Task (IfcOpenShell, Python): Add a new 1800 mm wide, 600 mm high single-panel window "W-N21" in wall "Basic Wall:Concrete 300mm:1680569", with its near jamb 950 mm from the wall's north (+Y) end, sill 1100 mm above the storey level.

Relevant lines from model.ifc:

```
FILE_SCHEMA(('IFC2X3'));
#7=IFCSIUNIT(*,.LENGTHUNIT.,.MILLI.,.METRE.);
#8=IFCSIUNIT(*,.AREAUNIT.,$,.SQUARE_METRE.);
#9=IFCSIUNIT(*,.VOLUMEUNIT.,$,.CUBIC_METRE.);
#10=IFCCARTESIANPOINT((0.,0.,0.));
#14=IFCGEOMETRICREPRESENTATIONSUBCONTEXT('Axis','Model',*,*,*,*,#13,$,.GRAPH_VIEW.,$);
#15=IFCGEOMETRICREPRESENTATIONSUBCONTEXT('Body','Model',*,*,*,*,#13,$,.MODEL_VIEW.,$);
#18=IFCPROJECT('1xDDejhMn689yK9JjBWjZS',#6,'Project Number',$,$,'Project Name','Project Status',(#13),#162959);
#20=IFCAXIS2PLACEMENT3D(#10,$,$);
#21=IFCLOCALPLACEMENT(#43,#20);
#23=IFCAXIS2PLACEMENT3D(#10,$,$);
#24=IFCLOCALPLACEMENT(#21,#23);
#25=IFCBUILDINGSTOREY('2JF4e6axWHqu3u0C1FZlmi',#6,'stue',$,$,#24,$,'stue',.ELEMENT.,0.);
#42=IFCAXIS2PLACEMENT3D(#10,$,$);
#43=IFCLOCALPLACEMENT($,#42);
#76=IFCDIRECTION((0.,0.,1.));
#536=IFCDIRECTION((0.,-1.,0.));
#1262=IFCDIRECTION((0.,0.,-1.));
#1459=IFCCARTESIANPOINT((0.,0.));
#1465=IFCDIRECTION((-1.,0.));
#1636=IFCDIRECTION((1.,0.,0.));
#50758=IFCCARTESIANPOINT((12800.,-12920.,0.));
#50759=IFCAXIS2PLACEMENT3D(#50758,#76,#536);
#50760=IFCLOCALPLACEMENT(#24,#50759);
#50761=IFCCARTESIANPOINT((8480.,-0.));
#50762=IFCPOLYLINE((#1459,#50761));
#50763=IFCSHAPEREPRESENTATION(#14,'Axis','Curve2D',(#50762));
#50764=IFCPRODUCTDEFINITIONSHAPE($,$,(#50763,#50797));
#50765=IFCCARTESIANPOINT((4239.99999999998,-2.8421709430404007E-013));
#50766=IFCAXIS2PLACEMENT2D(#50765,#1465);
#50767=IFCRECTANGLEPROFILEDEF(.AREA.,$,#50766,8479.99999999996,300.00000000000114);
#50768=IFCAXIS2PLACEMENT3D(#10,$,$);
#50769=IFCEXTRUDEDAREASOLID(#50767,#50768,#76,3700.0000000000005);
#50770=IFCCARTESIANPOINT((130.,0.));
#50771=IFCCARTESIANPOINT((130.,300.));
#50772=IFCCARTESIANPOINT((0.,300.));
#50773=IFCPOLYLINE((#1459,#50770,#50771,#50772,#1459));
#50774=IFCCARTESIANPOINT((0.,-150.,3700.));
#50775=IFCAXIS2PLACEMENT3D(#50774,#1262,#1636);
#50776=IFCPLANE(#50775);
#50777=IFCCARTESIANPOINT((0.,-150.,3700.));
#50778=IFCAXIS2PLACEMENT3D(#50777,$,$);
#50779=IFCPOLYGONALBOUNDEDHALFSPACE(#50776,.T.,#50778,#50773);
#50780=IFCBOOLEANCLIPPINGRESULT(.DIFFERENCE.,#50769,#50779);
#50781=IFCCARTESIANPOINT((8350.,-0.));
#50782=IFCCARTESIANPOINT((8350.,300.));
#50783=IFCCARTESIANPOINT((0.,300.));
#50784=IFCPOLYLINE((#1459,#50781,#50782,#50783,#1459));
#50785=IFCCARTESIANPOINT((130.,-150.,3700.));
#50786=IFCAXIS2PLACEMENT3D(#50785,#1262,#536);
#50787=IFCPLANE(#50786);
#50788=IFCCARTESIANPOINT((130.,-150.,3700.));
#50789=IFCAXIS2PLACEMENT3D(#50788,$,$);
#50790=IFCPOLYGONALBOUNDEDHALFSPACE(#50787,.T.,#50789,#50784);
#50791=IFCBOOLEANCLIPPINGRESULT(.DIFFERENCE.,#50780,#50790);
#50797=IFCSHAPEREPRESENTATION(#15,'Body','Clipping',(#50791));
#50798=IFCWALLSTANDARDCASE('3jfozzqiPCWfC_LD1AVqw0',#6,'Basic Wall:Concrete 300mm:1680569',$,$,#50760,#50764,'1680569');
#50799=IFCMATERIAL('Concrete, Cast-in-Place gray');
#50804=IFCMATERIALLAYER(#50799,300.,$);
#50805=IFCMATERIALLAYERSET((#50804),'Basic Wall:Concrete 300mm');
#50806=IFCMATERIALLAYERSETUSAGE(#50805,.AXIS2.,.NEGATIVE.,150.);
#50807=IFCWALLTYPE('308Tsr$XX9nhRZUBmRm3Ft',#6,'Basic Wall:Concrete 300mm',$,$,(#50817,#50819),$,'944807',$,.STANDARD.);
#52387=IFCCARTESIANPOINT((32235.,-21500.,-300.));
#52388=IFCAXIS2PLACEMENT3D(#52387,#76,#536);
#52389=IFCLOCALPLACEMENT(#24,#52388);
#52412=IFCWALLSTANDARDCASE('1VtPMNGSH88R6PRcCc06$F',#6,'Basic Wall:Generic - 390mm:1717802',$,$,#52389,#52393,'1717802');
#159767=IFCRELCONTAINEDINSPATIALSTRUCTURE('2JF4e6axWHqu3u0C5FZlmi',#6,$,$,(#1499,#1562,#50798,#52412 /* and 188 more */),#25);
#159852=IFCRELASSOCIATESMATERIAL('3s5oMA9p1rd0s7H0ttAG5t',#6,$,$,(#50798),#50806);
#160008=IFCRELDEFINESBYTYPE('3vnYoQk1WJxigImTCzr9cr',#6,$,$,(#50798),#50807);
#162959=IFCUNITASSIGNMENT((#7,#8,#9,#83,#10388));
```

```python
import numpy as np
import ifcopenshell
import ifcopenshell.api.feature
import ifcopenshell.api.geometry
import ifcopenshell.api.root
import ifcopenshell.api.spatial
import ifcopenshell.api.type
import ifcopenshell.geom
import ifcopenshell.util.element
import ifcopenshell.util.placement
import ifcopenshell.util.representation
import ifcopenshell.util.shape
import ifcopenshell.util.unit

model = ifcopenshell.open("model.ifc")
unit_scale = ifcopenshell.util.unit.calculate_unit_scale(model)
settings = ifcopenshell.geom.settings()


def volume(element):
    """Net volume in cubic metres, openings subtracted."""
    shape = ifcopenshell.geom.create_shape(settings, element)
    return ifcopenshell.util.shape.get_volume(shape.geometry)


wall = model.by_guid("3jfozzqiPCWfC_LD1AVqw0")
storey = ifcopenshell.util.element.get_container(wall, ifc_class="IfcBuildingStorey")
context = ifcopenshell.util.representation.get_context(model, "Model", "Body", "MODEL_VIEW")
before = volume(wall)

width, height, from_end, sill = 1.8, 0.6, 0.95, 1.1  # metres

# The wall runs along its own X axis, and the end named is its -X end.
wall_shape = ifcopenshell.geom.create_shape(settings, wall)
x, y, z = ifcopenshell.util.shape.get_vertices(wall_shape.geometry).T
start = x.min() + from_end
face, thickness = float(y.min()), float(y.max() - y.min())
wall_matrix = ifcopenshell.util.placement.get_local_placement(wall.ObjectPlacement)
level = ifcopenshell.util.placement.get_local_placement(storey.ObjectPlacement)[2, 3]


def in_wall(x, y):
    """Placement at x, y metres in the wall's axes, at sill height."""
    matrix = wall_matrix.copy()
    matrix[:, 3] = wall_matrix @ np.array([x / unit_scale, y / unit_scale, 0.0, 1.0])
    matrix[2, 3] = level + sill / unit_scale
    return matrix


# Opening: a box that overshoots both wall faces by 50 mm.
opening = ifcopenshell.api.root.create_entity(model, ifc_class="IfcOpeningElement")
box = ifcopenshell.api.geometry.add_wall_representation(
    model, context=context, length=width, height=height, thickness=thickness + 0.1
)
ifcopenshell.api.geometry.assign_representation(model, product=opening, representation=box)
ifcopenshell.api.geometry.edit_object_placement(model, product=opening, matrix=in_wall(start, face - 0.05), is_si=False)
ifcopenshell.api.feature.add_feature(model, feature=opening, element=wall)

window = ifcopenshell.api.root.create_entity(model, ifc_class="IfcWindow", name="W-N21")
window.OverallWidth, window.OverallHeight = width / unit_scale, height / unit_scale
body = ifcopenshell.api.geometry.add_window_representation(
    model,
    context=context,
    overall_width=window.OverallWidth,
    overall_height=window.OverallHeight,
    partition_type="SINGLE_PANEL",
)
ifcopenshell.api.geometry.assign_representation(model, product=window, representation=body)
ifcopenshell.api.spatial.assign_container(model, products=[window], relating_structure=storey)
fills = ifcopenshell.api.feature.add_filling(model, opening=opening, element=window)
fills.OwnerHistory = window.OwnerHistory  # required in IFC2X3

# IFC2X3 keeps the operation on the window style.
style = ifcopenshell.api.root.create_entity(model, ifc_class="IfcWindowStyle", name="W-N21")
style.OperationType, style.ConstructionType = "SINGLE_PANEL", "NOTDEFINED"
style.ParameterTakesPrecedence = style.Sizeable = False
ifcopenshell.api.type.assign_type(model, related_objects=[window], relating_type=style)

# Centre the window in the wall's thickness.
ifcopenshell.api.geometry.edit_object_placement(model, product=window, matrix=in_wall(start, face), is_si=False)
window_shape = ifcopenshell.geom.create_shape(settings, window)
depth = ifcopenshell.util.shape.get_vertices(window_shape.geometry)[:, 1]
offset = face + thickness / 2 - (depth.min() + depth.max()) / 2
ifcopenshell.api.geometry.edit_object_placement(model, product=window, matrix=in_wall(start, offset), is_si=False)

after = volume(wall)

print(f"wall volume {before:.3f} -> {after:.3f} m3")

model.write("model_rev.ifc")
```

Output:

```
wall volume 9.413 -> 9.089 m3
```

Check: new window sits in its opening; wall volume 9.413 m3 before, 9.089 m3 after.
